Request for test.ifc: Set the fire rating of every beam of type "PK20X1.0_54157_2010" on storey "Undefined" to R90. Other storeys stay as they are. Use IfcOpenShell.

First a look at what the model holds.

```python
import ifcopenshell
import ifcopenshell.util.element

model = ifcopenshell.open("test.ifc")
print(model.schema)
storey = next(s for s in model.by_type("IfcBuildingStorey") if s.Name == "Undefined")
beams = [e for e in ifcopenshell.util.element.get_decomposition(storey) if e.is_a("IfcBeam")]
seen = {}
for e in beams:
    element_type = ifcopenshell.util.element.get_type(e)
    key = (element_type.Name if element_type != e and element_type else None, ifcopenshell.util.element.get_pset(e, "Pset_BeamCommon", "FireRating"))
    seen[key] = seen.get(key, 0) + 1
for (name, value), count in sorted(seen.items(), key=str):
    print(count, "x", name, "|", value)
```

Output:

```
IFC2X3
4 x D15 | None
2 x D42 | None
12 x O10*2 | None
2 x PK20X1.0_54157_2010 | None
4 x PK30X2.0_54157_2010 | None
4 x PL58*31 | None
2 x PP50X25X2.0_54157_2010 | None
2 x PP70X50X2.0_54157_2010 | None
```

```python
import ifcopenshell
import ifcopenshell.api.pset
import ifcopenshell.util.element

model = ifcopenshell.open("test.ifc")

storey = next(s for s in model.by_type("IfcBuildingStorey") if s.Name == "Undefined")
beams = [e for e in ifcopenshell.util.element.get_decomposition(storey) if e.is_a("IfcBeam")]

count = 0
for e in beams:
    element_type = ifcopenshell.util.element.get_type(e)
    if element_type in (None, e) or element_type.Name != "PK20X1.0_54157_2010":
        continue
    found = ifcopenshell.util.element.get_pset(e, "Pset_BeamCommon", should_inherit=False)
    if found:
        pset = model.by_id(found["id"])
        if len(ifcopenshell.util.element.get_elements_by_pset(pset)) > 1:
            pset = ifcopenshell.api.pset.unshare_pset(model, products=[e], pset=pset)[0]
    else:
        pset = ifcopenshell.api.pset.add_pset(model, product=e, name="Pset_BeamCommon")
    ifcopenshell.api.pset.edit_pset(model, pset=pset, properties={"FireRating": "R90"})
    count += 1

print(count, "beams updated")

model.write("test_edited.ifc")
```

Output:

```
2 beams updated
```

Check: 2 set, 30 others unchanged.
